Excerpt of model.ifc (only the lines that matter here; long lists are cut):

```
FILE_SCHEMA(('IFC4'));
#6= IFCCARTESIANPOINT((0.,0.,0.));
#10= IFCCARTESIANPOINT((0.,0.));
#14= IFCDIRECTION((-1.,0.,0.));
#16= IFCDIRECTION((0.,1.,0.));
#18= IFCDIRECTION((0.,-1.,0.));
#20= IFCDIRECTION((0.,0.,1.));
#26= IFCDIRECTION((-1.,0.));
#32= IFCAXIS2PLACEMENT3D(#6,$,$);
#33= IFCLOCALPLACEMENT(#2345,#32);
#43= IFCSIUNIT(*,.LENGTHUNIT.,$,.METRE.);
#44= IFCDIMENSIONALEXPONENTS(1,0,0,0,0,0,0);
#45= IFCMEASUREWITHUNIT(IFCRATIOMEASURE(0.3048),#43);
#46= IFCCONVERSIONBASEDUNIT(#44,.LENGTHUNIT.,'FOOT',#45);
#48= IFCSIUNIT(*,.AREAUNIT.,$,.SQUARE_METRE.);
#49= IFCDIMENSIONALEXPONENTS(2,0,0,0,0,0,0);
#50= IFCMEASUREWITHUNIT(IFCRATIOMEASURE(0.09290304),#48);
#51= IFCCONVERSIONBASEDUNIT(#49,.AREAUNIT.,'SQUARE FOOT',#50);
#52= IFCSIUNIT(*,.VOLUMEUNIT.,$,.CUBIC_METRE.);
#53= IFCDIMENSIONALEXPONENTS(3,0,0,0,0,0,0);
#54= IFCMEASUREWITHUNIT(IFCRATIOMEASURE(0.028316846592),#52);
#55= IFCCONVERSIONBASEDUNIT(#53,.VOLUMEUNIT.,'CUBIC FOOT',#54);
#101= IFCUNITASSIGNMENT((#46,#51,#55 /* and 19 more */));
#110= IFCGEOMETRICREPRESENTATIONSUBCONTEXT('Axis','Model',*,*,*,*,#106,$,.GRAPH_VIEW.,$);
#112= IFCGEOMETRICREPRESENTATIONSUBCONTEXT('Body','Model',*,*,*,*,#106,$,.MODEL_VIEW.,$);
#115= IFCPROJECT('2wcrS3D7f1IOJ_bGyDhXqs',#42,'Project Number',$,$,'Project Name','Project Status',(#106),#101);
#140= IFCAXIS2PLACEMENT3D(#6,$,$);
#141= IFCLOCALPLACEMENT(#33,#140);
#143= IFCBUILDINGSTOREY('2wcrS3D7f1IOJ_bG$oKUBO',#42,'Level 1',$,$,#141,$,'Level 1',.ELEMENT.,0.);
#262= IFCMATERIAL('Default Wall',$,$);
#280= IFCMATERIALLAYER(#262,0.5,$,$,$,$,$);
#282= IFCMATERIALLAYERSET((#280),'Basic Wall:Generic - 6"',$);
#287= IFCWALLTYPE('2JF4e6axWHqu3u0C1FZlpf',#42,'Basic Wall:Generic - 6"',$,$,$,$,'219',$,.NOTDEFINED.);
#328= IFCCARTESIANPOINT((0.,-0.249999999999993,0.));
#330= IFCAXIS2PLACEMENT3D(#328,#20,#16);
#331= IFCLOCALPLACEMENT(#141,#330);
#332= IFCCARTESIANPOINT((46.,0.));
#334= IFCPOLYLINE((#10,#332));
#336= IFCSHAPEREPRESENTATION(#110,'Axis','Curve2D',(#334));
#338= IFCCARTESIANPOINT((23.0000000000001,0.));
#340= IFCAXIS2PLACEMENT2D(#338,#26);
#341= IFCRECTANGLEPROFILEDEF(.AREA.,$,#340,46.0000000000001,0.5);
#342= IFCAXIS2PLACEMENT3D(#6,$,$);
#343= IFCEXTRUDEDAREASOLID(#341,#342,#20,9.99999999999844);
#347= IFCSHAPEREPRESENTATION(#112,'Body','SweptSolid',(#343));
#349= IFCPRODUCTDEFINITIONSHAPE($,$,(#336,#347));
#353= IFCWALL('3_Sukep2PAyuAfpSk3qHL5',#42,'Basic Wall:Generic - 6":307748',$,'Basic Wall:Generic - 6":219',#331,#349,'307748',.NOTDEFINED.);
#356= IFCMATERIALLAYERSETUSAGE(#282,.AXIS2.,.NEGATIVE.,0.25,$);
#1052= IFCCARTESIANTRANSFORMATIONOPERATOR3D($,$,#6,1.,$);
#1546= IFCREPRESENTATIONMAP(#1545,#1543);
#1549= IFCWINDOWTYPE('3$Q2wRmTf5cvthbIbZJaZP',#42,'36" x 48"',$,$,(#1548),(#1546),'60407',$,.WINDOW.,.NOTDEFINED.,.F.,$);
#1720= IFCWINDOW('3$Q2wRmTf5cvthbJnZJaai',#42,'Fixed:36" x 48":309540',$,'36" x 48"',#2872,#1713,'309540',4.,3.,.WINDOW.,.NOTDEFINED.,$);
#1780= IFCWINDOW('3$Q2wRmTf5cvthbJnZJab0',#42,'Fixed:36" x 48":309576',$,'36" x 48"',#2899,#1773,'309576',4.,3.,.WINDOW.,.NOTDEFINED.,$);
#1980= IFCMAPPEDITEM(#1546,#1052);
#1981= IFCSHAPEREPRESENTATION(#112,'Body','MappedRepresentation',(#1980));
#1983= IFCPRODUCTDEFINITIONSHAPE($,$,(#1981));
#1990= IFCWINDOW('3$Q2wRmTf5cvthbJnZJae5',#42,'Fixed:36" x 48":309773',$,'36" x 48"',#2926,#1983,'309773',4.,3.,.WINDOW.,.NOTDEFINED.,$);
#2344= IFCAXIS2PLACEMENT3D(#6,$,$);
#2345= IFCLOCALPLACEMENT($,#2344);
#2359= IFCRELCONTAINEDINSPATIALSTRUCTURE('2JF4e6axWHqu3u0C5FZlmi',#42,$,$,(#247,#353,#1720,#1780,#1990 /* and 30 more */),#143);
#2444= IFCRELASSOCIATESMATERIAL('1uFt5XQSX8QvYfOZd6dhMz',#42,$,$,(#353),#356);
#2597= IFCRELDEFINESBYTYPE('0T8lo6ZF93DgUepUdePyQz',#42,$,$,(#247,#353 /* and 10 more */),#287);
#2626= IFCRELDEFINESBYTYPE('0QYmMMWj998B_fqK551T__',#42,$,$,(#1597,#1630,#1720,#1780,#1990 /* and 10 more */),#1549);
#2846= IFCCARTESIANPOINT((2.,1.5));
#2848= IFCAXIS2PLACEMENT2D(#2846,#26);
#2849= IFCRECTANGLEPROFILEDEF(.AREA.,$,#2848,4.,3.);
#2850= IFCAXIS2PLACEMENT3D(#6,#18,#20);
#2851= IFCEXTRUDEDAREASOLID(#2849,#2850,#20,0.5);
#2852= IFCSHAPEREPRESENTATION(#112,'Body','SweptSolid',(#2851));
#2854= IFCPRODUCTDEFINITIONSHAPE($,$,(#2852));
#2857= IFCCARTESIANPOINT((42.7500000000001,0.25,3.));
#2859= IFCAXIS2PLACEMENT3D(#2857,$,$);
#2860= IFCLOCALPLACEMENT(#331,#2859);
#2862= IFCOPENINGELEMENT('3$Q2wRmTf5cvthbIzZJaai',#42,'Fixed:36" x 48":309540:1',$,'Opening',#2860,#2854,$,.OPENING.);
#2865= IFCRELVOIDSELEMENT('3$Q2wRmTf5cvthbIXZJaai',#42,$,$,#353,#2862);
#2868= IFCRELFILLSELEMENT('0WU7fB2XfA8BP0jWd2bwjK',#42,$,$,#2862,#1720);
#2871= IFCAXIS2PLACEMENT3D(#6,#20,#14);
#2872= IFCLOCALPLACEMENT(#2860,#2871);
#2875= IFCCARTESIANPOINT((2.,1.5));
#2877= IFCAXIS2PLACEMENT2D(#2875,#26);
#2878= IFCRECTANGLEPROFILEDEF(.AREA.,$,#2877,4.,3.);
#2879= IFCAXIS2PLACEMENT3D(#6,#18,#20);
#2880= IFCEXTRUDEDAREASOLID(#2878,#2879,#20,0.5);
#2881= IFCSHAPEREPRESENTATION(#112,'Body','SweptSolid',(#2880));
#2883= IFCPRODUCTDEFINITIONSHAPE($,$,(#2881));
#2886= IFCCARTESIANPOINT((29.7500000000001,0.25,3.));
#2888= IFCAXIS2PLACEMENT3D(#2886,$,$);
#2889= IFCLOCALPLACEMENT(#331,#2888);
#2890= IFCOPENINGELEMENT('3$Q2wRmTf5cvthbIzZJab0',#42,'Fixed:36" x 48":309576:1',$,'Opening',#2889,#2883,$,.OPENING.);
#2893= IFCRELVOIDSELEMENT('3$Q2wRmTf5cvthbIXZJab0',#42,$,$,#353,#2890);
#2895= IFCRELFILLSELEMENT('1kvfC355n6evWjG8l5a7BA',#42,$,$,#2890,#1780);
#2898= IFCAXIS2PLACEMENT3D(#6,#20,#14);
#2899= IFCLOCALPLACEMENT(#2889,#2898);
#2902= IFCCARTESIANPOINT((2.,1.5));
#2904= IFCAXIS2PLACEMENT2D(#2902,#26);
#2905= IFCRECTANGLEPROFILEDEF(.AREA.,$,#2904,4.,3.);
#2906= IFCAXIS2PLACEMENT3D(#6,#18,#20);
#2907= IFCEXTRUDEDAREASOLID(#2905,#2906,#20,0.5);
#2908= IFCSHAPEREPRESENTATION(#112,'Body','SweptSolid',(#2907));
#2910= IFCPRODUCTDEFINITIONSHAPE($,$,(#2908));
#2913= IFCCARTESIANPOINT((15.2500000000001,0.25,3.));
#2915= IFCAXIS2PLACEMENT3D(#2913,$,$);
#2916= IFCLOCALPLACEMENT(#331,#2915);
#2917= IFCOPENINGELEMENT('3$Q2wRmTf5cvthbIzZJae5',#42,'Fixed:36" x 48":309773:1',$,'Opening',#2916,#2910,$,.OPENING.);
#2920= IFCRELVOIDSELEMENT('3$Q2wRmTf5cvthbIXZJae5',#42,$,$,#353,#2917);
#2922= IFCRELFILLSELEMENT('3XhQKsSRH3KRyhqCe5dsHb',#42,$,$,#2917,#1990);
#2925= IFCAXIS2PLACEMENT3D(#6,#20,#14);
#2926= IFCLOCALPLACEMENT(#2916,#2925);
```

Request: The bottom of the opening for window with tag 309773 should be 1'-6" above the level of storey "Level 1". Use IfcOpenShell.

```python
import numpy as np
import ifcopenshell
import ifcopenshell.api.geometry
import ifcopenshell.geom
import ifcopenshell.util.element
import ifcopenshell.util.placement
import ifcopenshell.util.shape
import ifcopenshell.util.unit

model = ifcopenshell.open("model.ifc")
unit_scale = ifcopenshell.util.unit.calculate_unit_scale(model)

window = model.by_guid("3$Q2wRmTf5cvthbJnZJae5")
opening = window.FillsVoids[0].RelatingOpeningElement
storey = ifcopenshell.util.element.get_container(window, ifc_class="IfcBuildingStorey")
level = ifcopenshell.util.placement.get_local_placement(storey.ObjectPlacement)[2, 3]

# The opening's origin need not be at the sill, so measure its lowest point.
shape = ifcopenshell.geom.create_shape(ifcopenshell.geom.settings(), opening)
bottom = ifcopenshell.util.shape.get_shape_bottom_elevation(shape, shape.geometry) / unit_scale
dz = level + 18 * 0.0254 / unit_scale - bottom

shift = np.array([0.0, 0.0, dz])
# The window is placed relative to its opening, so it follows when the opening moves.
matrix = ifcopenshell.util.placement.get_local_placement(opening.ObjectPlacement)
matrix[:3, 3] += shift
ifcopenshell.api.geometry.edit_object_placement(
    model, product=opening, matrix=matrix, is_si=False, should_transform_children=True
)

print(f"moved by {dz * unit_scale:+.3f} m")

model.write("model_v2.ifc")
```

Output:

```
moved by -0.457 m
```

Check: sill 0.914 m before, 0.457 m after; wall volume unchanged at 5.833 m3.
